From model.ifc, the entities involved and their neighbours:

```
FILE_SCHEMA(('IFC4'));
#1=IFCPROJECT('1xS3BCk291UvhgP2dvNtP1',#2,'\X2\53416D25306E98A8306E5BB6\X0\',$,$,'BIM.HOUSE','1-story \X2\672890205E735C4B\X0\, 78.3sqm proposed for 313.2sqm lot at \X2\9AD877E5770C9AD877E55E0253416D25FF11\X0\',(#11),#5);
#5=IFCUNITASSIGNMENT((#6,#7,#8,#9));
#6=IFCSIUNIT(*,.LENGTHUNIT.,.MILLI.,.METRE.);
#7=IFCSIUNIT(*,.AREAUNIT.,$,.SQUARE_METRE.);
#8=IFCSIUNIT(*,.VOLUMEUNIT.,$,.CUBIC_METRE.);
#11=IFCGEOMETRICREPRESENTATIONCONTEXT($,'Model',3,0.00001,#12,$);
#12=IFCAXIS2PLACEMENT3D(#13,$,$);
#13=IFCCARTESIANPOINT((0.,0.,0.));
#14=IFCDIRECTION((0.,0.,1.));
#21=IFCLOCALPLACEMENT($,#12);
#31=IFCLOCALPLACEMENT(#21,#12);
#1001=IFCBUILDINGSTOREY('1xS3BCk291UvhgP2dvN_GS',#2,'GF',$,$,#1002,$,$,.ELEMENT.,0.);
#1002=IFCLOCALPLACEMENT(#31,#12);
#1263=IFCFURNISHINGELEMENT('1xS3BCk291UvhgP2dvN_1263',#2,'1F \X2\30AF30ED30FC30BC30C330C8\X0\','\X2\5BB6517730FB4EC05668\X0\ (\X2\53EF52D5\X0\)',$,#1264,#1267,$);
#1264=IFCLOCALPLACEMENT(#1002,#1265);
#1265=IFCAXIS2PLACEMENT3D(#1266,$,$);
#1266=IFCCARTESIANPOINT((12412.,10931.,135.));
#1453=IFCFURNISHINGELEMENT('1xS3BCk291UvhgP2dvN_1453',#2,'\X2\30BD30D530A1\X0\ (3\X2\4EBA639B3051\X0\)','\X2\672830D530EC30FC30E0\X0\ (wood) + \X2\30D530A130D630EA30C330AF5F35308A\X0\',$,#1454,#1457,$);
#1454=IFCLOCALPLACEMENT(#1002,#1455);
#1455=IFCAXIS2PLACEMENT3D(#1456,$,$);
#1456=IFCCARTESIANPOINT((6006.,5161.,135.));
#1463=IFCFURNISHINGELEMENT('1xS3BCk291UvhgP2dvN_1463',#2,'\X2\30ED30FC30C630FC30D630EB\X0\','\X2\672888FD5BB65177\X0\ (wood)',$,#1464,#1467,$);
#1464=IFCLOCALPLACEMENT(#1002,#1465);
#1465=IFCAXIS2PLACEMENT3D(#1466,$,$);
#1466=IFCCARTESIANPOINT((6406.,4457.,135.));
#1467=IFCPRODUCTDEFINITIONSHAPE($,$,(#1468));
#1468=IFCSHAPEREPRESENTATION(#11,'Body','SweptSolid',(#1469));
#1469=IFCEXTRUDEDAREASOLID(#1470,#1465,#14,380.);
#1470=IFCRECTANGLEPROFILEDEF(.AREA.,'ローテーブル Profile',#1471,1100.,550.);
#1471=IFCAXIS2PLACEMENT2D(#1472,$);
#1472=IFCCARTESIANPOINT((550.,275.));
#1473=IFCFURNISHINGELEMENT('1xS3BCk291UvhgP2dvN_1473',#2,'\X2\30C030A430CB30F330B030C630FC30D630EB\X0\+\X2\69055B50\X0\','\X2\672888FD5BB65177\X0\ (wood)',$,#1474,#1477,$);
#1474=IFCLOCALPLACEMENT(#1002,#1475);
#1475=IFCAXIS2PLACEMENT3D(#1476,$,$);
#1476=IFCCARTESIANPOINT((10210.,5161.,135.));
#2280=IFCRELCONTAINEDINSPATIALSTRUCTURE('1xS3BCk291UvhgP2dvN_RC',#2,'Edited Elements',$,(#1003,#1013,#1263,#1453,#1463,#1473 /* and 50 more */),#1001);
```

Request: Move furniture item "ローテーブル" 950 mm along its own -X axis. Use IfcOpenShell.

```python
import ifcopenshell
import ifcopenshell.api.geometry
import ifcopenshell.util.placement
import ifcopenshell.util.unit

model = ifcopenshell.open("model.ifc")
unit_scale = ifcopenshell.util.unit.calculate_unit_scale(model)

item = model.by_id(1463)
matrix = ifcopenshell.util.placement.get_local_placement(item.ObjectPlacement)
matrix[:3, 3] -= matrix[:3, 0] * 0.95 / unit_scale
ifcopenshell.api.geometry.edit_object_placement(model, product=item, matrix=matrix, is_si=False)

print(ifcopenshell.util.placement.get_local_placement(item.ObjectPlacement).round(3) + 0.0)

model.write("model_rev.ifc")
```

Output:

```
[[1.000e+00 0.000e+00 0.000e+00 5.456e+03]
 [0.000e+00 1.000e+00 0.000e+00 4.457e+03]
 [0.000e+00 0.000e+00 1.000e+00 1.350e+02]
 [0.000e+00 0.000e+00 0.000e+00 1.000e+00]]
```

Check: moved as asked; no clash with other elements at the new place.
